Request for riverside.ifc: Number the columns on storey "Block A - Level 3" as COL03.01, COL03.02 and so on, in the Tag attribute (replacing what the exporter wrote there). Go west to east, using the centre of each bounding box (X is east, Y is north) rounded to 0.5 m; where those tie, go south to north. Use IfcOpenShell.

First a look at what the model holds.

```python
import ifcopenshell
import ifcopenshell.util.element
import ifcopenshell.util.placement

model = ifcopenshell.open("riverside.ifc")
print(model.schema)
storey = next(s for s in model.by_type("IfcBuildingStorey") if s.Name == "Block A - Level 3")
columns = [e for e in ifcopenshell.util.element.get_decomposition(storey) if e.is_a("IfcColumn")]
for e in sorted(columns, key=lambda e: e.id()):
    origin = ifcopenshell.util.placement.get_local_placement(e.ObjectPlacement)[:3, 3]
    print(e.id(), e.Tag, e.Name, origin.round(2) + 0.0, sep=" | ")
```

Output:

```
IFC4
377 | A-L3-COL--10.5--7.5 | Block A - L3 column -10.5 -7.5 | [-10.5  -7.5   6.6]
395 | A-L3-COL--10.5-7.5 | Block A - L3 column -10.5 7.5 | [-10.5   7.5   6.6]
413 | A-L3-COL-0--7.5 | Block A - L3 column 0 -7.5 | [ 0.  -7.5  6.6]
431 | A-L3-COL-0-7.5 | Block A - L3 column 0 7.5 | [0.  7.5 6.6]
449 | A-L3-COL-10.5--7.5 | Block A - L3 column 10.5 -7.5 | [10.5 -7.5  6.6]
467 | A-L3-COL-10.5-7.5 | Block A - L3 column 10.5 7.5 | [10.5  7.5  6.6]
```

```python
import ifcopenshell
import ifcopenshell.geom
import ifcopenshell.util.element
import ifcopenshell.util.shape

model = ifcopenshell.open("riverside.ifc")
settings = ifcopenshell.geom.settings()
settings.set("use-world-coords", True)


def centre(element):
    shape = ifcopenshell.geom.create_shape(settings, element)
    return ifcopenshell.util.shape.get_bbox_centroid(shape.geometry)


storey = next(s for s in model.by_type("IfcBuildingStorey") if s.Name == "Block A - Level 3")
columns = [e for e in ifcopenshell.util.element.get_decomposition(storey) if e.is_a("IfcColumn")]

# Insertion points can sit at a corner or the storey origin, so sort by the geometry (in metres).
centres = {e: centre(e) for e in columns}
columns.sort(key=lambda e: (round(centres[e][0] / 0.5), centres[e][1]))

for i, e in enumerate(columns, start=1):
    number = f"COL03.{i:02d}"
    e.Tag = number
    print(e.id(), number)

model.write("riverside_v2.ifc")
```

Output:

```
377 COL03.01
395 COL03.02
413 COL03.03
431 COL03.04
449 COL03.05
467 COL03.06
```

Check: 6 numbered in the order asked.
